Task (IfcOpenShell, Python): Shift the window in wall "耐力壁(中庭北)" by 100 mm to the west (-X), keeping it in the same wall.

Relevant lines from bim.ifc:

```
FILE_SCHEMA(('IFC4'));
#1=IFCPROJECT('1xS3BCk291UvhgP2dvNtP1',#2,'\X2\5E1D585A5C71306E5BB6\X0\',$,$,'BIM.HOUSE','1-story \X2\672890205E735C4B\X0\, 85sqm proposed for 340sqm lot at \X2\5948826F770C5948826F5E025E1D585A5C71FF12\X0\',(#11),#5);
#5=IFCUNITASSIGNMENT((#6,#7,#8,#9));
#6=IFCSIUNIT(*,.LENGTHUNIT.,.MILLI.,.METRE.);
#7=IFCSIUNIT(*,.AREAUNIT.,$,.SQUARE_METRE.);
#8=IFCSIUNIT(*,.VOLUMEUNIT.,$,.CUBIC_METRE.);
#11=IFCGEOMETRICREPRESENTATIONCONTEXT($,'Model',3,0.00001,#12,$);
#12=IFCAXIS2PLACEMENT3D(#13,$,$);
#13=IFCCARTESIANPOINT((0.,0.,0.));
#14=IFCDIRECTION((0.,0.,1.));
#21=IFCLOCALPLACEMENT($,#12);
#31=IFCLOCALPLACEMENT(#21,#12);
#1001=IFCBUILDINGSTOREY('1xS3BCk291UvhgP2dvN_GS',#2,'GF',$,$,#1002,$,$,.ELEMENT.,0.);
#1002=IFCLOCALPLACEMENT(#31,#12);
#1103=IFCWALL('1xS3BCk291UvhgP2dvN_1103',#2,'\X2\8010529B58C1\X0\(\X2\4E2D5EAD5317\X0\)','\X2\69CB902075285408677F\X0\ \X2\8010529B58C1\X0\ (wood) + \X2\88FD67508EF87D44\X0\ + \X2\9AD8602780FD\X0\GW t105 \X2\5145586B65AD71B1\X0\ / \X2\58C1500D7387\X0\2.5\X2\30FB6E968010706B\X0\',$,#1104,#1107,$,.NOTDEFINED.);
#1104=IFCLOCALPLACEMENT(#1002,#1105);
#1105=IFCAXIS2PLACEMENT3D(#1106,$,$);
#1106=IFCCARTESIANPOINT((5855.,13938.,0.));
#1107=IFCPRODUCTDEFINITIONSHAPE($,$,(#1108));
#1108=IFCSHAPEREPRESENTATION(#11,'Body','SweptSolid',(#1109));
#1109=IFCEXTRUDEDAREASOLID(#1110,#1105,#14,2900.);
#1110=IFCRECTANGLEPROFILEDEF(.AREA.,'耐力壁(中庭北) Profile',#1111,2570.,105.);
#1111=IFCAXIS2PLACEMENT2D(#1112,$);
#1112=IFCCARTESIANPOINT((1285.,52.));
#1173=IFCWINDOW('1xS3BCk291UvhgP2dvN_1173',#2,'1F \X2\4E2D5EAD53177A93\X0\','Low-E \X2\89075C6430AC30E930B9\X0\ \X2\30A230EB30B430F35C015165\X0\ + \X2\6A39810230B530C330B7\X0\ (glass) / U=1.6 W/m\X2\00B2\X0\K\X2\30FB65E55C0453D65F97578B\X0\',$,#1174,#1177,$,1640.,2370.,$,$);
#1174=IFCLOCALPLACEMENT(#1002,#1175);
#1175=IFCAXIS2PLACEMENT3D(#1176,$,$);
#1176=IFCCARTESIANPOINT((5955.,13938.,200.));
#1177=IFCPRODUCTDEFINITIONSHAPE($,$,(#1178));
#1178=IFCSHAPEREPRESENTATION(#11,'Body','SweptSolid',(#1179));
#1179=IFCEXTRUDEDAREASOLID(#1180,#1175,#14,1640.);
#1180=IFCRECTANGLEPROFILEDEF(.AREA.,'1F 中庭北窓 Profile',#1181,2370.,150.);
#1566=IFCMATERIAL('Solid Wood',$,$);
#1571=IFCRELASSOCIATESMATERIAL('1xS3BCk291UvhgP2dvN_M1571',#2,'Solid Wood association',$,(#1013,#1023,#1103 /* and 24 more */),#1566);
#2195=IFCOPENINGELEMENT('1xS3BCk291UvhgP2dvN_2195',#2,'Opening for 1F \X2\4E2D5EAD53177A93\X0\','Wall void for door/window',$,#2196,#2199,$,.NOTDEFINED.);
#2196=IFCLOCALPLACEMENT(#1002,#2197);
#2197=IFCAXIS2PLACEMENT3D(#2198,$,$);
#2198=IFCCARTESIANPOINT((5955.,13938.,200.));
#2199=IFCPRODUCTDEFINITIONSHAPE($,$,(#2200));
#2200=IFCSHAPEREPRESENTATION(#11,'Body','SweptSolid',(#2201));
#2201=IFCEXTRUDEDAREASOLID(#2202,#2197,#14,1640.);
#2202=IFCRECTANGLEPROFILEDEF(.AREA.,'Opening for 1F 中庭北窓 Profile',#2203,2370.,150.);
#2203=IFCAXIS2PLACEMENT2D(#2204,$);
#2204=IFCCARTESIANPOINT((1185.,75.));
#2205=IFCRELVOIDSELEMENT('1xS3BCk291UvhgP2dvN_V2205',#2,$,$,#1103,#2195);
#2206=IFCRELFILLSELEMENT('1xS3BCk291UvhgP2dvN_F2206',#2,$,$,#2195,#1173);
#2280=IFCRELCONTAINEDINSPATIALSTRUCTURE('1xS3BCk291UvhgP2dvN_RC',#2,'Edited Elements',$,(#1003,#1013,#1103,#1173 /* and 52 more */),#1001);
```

```python
import ifcopenshell
import ifcopenshell.api.geometry
import ifcopenshell.util.placement

model = ifcopenshell.open("bim.ifc")

window = model.by_guid("1xS3BCk291UvhgP2dvN_1173")
opening = window.FillsVoids[0].RelatingOpeningElement
wall = opening.VoidsElements[0].RelatingBuildingElement

wall_matrix = ifcopenshell.util.placement.get_local_placement(wall.ObjectPlacement)
shift = wall_matrix[:3, 0] * -100.0
before = ifcopenshell.util.placement.get_local_placement(window.ObjectPlacement)[:3, 3].copy()

# The window is not placed relative to its opening, so move both.
for product in (opening, window):
    matrix = ifcopenshell.util.placement.get_local_placement(product.ObjectPlacement)
    matrix[:3, 3] += shift
    ifcopenshell.api.geometry.edit_object_placement(model, product=product, matrix=matrix, is_si=False)

after = ifcopenshell.util.placement.get_local_placement(window.ObjectPlacement)[:3, 3]
print("window moved by", (after - before).round(3) + 0.0)

model.write("bim_rev.ifc")
```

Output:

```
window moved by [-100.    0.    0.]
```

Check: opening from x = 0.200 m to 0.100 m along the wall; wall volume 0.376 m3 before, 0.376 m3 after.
